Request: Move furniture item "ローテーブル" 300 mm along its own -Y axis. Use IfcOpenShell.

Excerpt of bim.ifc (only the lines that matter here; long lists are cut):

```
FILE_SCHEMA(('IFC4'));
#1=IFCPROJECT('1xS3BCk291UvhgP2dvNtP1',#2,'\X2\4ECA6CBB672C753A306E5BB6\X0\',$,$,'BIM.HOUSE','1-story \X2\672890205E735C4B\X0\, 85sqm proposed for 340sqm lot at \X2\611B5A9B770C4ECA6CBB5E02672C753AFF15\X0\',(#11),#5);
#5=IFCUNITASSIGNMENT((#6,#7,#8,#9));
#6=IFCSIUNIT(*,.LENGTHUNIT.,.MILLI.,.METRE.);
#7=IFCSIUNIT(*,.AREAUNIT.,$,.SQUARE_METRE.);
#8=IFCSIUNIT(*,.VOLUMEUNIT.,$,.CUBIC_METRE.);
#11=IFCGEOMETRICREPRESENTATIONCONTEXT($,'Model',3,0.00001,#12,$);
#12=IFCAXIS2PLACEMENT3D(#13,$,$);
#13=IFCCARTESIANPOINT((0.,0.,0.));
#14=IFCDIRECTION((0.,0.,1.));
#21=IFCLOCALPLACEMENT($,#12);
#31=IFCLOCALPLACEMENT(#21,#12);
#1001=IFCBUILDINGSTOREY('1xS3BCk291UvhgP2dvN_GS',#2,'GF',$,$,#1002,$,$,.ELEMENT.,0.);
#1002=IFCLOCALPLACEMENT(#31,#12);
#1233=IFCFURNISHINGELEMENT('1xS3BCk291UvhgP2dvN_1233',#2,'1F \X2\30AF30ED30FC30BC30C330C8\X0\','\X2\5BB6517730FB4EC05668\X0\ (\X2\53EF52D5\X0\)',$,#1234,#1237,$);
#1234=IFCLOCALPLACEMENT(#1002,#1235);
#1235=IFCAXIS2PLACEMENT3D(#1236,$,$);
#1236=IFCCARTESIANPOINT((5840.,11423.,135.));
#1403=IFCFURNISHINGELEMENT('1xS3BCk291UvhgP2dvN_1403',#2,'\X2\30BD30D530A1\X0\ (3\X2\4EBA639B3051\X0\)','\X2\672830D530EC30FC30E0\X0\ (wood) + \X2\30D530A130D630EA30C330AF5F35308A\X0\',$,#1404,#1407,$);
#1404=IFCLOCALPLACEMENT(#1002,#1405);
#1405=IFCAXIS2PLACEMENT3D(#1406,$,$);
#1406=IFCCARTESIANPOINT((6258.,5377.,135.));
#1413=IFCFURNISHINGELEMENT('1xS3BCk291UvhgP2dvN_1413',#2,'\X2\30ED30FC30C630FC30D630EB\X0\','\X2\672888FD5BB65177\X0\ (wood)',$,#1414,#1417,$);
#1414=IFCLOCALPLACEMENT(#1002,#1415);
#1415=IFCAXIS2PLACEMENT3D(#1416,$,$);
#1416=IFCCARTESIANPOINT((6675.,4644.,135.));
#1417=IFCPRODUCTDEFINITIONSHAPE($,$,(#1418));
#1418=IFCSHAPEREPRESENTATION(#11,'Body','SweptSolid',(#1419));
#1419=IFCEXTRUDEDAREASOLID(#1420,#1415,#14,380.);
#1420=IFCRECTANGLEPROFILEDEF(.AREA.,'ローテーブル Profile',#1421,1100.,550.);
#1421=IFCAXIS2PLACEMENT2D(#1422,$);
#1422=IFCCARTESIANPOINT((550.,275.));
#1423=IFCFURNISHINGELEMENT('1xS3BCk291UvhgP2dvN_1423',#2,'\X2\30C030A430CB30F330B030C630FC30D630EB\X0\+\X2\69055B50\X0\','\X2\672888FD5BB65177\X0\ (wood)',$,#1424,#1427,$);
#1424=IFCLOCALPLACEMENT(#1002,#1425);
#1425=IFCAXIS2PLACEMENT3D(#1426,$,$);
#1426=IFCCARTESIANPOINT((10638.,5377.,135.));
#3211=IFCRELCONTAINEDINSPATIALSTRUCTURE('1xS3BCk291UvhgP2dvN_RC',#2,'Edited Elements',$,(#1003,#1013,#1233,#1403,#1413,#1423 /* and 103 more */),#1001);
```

```python
import ifcopenshell
import ifcopenshell.api.geometry
import ifcopenshell.util.placement
import ifcopenshell.util.unit

model = ifcopenshell.open("bim.ifc")
unit_scale = ifcopenshell.util.unit.calculate_unit_scale(model)

item = model.by_guid("1xS3BCk291UvhgP2dvN_1413")
matrix = ifcopenshell.util.placement.get_local_placement(item.ObjectPlacement)
matrix[:3, 3] -= matrix[:3, 1] * 0.3 / unit_scale
ifcopenshell.api.geometry.edit_object_placement(model, product=item, matrix=matrix, is_si=False)

print(ifcopenshell.util.placement.get_local_placement(item.ObjectPlacement).round(3) + 0.0)

model.write("bim-out.ifc")
```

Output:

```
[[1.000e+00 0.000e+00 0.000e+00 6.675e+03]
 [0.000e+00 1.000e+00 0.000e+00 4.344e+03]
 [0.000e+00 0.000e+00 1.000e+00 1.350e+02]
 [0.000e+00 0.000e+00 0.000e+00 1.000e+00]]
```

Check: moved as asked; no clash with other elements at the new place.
